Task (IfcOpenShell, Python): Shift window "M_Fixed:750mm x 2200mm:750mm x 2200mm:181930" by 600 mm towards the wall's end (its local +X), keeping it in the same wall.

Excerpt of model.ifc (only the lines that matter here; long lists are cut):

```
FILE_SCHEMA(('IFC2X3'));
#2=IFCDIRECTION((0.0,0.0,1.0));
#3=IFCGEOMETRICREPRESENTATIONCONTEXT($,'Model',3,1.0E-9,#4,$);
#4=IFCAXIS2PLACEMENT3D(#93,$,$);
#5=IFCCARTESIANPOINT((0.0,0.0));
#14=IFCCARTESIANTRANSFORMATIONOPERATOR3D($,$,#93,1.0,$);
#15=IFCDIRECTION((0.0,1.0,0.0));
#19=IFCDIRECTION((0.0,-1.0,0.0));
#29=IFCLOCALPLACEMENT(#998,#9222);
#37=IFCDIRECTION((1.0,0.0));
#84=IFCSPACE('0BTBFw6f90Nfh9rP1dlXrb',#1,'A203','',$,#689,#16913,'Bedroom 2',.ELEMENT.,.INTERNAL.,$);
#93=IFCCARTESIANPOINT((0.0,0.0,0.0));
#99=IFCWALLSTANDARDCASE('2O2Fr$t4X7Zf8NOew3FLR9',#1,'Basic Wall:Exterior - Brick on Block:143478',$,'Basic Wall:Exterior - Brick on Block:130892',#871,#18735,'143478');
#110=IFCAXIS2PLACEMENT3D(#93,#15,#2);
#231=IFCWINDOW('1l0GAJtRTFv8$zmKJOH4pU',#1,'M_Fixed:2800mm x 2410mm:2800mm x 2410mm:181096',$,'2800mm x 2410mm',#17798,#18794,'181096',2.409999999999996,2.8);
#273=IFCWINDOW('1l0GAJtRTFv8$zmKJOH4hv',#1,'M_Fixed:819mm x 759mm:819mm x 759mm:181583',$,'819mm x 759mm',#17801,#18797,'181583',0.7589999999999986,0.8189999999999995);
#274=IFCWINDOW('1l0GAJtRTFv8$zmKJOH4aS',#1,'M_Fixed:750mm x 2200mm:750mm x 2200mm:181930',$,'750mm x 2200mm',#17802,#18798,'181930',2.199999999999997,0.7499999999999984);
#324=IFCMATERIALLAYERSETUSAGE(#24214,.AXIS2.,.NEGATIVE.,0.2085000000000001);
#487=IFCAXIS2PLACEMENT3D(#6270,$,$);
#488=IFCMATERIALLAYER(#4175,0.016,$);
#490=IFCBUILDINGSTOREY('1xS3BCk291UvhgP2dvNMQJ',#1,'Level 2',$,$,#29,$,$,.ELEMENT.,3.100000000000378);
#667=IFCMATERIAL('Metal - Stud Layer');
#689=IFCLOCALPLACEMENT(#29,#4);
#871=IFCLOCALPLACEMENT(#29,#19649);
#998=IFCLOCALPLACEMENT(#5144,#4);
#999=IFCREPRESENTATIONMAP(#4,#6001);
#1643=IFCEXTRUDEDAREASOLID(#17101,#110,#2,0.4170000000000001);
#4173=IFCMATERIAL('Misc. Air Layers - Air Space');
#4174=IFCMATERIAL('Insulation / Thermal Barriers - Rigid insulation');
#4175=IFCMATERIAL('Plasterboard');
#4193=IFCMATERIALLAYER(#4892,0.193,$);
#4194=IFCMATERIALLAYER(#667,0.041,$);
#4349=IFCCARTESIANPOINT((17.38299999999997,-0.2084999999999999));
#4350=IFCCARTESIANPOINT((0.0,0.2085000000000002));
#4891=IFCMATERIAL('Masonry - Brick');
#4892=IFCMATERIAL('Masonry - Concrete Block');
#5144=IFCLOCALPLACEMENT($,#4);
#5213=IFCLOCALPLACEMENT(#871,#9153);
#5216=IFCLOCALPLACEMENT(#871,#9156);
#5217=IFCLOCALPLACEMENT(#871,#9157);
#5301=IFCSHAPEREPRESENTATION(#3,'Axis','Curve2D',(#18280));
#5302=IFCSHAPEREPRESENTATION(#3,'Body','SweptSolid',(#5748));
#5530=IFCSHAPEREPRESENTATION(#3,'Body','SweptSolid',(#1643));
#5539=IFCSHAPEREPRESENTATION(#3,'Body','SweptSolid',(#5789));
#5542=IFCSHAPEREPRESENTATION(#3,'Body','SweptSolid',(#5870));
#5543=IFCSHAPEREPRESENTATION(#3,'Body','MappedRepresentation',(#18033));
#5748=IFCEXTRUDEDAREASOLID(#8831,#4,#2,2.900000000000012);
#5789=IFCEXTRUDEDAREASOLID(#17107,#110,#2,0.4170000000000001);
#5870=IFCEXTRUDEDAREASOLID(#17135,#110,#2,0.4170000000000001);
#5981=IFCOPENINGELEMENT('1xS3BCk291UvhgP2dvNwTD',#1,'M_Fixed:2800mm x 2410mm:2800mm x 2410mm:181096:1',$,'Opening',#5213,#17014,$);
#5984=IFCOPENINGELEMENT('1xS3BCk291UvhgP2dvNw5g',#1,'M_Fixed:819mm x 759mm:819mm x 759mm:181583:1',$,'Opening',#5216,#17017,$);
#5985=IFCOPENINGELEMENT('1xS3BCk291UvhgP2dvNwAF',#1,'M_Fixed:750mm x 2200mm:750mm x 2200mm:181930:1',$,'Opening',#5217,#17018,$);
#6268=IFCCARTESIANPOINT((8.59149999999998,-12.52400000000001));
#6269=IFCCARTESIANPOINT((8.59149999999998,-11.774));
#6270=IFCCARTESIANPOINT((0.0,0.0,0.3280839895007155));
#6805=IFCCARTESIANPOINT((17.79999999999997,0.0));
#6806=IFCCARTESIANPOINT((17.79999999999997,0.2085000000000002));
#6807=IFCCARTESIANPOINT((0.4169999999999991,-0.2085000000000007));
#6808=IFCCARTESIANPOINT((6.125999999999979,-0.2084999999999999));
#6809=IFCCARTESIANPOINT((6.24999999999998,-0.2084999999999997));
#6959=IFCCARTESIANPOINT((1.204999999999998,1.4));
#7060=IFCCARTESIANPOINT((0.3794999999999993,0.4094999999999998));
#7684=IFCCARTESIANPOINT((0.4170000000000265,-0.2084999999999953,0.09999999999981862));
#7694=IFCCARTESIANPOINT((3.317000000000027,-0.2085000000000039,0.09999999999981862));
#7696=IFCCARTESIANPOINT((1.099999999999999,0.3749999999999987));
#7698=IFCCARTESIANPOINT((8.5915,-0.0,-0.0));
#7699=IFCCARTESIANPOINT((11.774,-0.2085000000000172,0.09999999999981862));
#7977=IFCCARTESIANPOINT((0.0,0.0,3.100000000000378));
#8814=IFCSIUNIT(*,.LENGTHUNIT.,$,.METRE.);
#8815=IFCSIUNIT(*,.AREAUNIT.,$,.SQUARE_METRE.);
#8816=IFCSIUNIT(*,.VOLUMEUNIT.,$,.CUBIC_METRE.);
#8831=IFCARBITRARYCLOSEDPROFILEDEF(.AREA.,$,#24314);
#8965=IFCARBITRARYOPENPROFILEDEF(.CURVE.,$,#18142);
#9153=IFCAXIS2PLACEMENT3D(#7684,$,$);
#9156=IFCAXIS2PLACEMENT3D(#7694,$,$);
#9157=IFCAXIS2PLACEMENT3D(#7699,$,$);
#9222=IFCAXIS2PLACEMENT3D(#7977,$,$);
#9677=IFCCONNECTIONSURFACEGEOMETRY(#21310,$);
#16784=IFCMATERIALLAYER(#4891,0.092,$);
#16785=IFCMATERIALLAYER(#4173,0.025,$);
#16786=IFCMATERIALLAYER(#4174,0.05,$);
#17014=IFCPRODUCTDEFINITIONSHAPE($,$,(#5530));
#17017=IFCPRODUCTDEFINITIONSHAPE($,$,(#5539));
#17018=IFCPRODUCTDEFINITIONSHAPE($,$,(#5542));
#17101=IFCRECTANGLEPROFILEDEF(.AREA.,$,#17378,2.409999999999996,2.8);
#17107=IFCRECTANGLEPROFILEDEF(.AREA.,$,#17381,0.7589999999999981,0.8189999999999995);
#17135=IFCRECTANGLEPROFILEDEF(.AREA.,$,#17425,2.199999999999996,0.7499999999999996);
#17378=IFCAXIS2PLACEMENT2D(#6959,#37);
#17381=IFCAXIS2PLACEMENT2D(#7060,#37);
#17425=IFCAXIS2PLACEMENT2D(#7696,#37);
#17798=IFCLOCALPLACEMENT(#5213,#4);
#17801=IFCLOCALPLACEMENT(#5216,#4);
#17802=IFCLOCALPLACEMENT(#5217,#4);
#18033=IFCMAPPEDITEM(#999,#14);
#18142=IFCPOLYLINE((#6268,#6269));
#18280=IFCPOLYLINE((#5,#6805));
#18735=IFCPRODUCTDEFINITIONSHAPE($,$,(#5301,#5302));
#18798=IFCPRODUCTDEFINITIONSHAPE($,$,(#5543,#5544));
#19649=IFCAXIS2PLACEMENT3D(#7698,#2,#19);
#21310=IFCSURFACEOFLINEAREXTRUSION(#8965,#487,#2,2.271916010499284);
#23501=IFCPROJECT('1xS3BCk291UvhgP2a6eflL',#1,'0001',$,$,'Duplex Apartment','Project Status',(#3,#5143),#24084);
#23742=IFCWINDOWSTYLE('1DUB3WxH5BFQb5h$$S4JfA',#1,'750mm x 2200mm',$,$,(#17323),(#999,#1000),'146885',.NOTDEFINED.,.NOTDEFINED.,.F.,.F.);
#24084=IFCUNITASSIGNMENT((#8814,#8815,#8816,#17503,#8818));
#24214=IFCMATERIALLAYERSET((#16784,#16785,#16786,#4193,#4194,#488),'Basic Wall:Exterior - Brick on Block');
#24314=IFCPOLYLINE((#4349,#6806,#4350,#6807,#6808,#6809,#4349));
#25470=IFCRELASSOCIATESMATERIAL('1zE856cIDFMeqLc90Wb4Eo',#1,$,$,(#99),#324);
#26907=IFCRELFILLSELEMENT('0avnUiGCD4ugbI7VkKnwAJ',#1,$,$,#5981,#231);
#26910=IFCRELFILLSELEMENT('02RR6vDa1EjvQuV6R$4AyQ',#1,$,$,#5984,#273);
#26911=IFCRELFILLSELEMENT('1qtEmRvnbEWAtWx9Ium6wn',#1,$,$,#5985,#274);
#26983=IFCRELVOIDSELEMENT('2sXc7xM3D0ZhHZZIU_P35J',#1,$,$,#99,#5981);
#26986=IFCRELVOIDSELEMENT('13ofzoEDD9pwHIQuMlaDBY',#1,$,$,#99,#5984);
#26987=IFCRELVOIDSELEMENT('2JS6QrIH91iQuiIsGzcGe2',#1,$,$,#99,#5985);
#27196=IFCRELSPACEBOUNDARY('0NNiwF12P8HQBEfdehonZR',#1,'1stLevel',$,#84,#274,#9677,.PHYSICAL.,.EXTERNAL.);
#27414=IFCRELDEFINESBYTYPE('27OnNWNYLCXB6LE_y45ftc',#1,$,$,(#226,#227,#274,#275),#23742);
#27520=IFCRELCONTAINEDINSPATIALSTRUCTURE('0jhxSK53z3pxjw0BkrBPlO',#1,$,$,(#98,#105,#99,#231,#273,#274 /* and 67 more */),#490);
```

```python
import numpy as np
import ifcopenshell
import ifcopenshell.api.geometry
import ifcopenshell.util.placement

model = ifcopenshell.open("model.ifc")

window = model.by_guid("1l0GAJtRTFv8$zmKJOH4aS")
opening = window.FillsVoids[0].RelatingOpeningElement
wall = opening.VoidsElements[0].RelatingBuildingElement

wall_matrix = ifcopenshell.util.placement.get_local_placement(wall.ObjectPlacement)
shift = wall_matrix[:3, 0] * 0.6
before = ifcopenshell.util.placement.get_local_placement(window.ObjectPlacement)[:3, 3].copy()

# The window is placed relative to its opening, so it follows when the opening moves.
matrix = ifcopenshell.util.placement.get_local_placement(opening.ObjectPlacement)
matrix[:3, 3] += shift
ifcopenshell.api.geometry.edit_object_placement(
    model, product=opening, matrix=matrix, is_si=False, should_transform_children=True
)

# Space boundary surfaces are stored in each space's coordinates; move them too.
for rel in window.ProvidesBoundaries:
    if not rel.ConnectionGeometry:
        continue
    surface = rel.ConnectionGeometry.SurfaceOnRelatingElement
    space_matrix = ifcopenshell.util.placement.get_local_placement(rel.RelatingSpace.ObjectPlacement)
    point = np.array(surface.Position.Location.Coordinates) + space_matrix[:3, :3].T @ shift
    surface.Position = model.createIfcAxis2Placement3D(
        model.createIfcCartesianPoint(point.tolist()), surface.Position.Axis, surface.Position.RefDirection
    )

after = ifcopenshell.util.placement.get_local_placement(window.ObjectPlacement)[:3, 3]
print("window moved by", (after - before).round(3) + 0.0)

model.write("model_edited.ifc")
```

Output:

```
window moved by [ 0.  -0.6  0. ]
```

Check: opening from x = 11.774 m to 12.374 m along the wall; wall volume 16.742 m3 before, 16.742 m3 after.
